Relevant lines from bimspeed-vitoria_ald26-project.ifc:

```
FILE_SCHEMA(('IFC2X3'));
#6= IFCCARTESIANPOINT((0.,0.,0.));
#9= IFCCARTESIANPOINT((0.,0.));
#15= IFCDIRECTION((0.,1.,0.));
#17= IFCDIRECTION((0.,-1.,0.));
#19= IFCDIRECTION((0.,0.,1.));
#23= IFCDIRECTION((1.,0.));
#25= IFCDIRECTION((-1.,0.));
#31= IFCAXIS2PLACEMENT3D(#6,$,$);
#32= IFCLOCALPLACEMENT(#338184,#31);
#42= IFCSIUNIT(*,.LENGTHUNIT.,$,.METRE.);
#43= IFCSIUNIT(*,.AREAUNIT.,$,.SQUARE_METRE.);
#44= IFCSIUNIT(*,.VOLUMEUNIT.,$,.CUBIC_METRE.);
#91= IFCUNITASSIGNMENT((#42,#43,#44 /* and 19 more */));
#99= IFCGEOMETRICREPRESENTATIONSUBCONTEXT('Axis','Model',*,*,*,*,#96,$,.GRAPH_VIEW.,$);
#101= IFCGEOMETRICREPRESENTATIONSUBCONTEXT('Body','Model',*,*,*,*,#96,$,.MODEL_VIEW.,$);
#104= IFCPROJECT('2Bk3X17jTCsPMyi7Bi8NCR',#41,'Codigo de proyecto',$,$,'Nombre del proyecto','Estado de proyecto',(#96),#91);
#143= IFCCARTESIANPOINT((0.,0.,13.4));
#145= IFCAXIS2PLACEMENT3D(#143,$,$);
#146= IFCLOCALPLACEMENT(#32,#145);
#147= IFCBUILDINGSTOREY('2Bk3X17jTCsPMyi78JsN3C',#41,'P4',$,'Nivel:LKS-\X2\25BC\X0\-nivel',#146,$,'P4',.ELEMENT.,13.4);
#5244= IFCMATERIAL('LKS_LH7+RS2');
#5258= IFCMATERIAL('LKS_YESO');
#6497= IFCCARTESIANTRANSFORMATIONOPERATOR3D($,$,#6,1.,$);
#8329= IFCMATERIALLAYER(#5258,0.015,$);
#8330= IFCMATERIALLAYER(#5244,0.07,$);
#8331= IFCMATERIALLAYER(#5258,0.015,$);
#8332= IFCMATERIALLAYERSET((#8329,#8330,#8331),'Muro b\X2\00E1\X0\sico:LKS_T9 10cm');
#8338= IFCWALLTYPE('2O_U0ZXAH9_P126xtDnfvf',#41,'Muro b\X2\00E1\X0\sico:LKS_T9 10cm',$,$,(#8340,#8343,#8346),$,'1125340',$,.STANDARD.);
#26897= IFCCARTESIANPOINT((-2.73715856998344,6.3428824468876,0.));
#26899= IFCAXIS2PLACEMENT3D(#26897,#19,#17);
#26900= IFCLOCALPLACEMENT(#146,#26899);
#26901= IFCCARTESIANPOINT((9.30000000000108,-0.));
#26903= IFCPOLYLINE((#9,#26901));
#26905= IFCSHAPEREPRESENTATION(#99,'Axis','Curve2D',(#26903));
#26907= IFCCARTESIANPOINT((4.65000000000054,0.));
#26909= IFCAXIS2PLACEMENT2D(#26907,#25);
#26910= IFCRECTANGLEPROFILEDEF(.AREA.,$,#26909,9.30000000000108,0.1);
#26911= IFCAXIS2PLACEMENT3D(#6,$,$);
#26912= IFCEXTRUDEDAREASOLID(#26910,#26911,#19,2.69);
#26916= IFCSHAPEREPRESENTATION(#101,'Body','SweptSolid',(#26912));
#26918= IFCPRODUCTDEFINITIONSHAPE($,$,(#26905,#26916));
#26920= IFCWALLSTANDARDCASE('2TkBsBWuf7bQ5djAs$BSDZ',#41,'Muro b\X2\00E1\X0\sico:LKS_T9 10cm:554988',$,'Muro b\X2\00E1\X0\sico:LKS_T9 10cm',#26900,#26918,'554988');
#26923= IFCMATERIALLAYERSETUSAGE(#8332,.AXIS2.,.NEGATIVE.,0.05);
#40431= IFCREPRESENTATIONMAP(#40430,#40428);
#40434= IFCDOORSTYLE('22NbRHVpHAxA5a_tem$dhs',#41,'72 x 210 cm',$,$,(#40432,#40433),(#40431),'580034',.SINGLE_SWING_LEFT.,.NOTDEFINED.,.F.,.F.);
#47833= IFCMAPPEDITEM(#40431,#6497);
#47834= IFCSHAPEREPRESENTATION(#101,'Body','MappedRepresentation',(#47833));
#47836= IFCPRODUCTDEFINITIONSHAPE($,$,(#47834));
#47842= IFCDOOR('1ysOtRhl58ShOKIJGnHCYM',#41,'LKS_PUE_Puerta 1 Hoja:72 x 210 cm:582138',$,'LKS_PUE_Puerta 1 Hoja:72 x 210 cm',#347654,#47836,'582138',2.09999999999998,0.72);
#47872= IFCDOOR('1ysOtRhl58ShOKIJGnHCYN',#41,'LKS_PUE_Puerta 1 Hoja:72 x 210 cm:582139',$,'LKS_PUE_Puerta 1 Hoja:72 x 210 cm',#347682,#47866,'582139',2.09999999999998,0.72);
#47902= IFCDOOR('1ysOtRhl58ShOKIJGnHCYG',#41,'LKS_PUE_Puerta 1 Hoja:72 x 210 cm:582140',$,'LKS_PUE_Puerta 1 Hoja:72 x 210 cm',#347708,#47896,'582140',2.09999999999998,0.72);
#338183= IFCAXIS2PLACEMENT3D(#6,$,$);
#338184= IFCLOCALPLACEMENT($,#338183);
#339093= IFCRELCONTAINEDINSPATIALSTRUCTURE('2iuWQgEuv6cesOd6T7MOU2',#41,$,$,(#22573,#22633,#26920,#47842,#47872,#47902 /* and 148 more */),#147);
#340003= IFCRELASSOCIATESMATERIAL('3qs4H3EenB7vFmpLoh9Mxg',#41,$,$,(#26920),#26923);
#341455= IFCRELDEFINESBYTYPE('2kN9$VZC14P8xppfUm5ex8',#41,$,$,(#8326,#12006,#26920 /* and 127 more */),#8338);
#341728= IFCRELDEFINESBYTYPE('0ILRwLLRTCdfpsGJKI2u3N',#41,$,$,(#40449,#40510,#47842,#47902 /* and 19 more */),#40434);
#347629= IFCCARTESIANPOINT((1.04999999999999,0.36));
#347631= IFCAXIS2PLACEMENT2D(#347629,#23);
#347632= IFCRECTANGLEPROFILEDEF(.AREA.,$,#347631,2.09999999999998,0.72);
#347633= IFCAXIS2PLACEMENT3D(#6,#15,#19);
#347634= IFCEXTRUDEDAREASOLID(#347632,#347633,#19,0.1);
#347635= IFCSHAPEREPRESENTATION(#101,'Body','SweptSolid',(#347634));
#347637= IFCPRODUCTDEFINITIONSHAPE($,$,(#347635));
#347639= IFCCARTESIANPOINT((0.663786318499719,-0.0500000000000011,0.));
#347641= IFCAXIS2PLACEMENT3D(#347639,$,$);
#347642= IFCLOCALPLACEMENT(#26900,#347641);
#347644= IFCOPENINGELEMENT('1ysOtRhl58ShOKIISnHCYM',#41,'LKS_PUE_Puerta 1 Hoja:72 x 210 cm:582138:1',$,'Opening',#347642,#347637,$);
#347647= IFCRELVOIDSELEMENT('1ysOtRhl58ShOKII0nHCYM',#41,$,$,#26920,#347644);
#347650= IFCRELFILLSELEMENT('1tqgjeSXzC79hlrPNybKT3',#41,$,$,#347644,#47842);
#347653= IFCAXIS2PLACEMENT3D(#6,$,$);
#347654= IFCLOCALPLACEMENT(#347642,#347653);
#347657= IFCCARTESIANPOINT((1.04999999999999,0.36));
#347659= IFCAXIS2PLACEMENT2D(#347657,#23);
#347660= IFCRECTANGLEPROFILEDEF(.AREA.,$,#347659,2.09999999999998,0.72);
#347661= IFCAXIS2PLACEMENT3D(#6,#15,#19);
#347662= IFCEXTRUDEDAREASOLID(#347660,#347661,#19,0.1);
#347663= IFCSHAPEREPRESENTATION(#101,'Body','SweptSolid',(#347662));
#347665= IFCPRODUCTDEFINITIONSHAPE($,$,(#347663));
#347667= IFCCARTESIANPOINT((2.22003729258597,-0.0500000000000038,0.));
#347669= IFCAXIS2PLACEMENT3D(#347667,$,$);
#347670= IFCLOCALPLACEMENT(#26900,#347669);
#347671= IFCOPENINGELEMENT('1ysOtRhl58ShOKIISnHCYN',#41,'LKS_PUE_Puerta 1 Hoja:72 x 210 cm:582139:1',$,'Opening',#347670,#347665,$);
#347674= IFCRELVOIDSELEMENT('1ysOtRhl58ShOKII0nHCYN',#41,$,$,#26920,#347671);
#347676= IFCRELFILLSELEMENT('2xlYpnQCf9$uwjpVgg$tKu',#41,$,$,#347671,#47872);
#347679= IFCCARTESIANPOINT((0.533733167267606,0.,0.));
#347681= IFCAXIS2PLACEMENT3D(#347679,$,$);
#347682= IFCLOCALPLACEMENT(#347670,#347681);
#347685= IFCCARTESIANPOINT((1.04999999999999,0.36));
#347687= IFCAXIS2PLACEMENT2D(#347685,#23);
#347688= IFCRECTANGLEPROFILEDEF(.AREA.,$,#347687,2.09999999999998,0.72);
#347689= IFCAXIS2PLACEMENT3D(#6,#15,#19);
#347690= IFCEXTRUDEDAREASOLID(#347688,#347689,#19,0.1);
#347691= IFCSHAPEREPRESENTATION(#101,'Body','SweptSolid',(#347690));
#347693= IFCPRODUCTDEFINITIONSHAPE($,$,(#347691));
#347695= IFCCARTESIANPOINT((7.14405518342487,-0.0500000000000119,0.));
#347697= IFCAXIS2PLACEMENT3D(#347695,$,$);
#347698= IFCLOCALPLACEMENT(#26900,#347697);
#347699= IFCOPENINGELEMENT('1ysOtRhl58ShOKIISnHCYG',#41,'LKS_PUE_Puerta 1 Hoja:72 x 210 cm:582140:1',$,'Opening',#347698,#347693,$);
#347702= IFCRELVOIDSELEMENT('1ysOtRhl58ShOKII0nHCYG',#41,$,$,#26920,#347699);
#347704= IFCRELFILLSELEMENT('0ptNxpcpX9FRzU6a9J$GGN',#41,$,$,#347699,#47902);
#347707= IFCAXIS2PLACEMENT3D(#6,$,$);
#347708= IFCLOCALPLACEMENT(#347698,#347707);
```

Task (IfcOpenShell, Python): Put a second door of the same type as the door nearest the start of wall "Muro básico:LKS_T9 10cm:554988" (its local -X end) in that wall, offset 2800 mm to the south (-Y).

```python
import ifcopenshell
import ifcopenshell.api.feature
import ifcopenshell.api.geometry
import ifcopenshell.api.root
import ifcopenshell.geom
import ifcopenshell.util.element
import ifcopenshell.util.placement
import ifcopenshell.util.shape

model = ifcopenshell.open("bimspeed-vitoria_ald26-project.ifc")
settings = ifcopenshell.geom.settings()


def volume(element):
    """Net volume in cubic metres, openings subtracted."""
    shape = ifcopenshell.geom.create_shape(settings, element)
    return ifcopenshell.util.shape.get_volume(shape.geometry)


def reuse_history(source, copy):
    """copy_class also copies each property set's owner history, people and application; keep the originals."""
    for rel in copy.IsDefinedBy:
        if rel.is_a("IfcRelDefinesByProperties") and (history := rel.RelatingPropertyDefinition.OwnerHistory):
            rel.RelatingPropertyDefinition.OwnerHistory = source.OwnerHistory
            ifcopenshell.util.element.remove_deep2(model, history)


door = model.by_id(47842)
opening = door.FillsVoids[0].RelatingOpeningElement
wall = opening.VoidsElements[0].RelatingBuildingElement
before = volume(wall)
shift = ifcopenshell.util.placement.get_local_placement(wall.ObjectPlacement)[:3, 0] * 2.8

# copy_class copies the void relationship, type, container and properties, but no geometry.
new_opening = ifcopenshell.api.root.copy_class(model, product=opening)
new_opening.Representation = ifcopenshell.util.element.copy_deep(
    model, opening.Representation, exclude=["IfcGeometricRepresentationContext", "IfcRepresentationMap"]
)
new_opening.Name = "LKS_PUE_Puerta 1 Hoja:72 x 210 cm"
new_door = ifcopenshell.api.root.copy_class(model, product=door)
new_door.Representation = ifcopenshell.util.element.copy_deep(
    model, door.Representation, exclude=["IfcGeometricRepresentationContext", "IfcRepresentationMap"]
)
new_door.Name = "LKS_PUE_Puerta 1 Hoja:72 x 210 cm"
new_door.Tag = None
reuse_history(door, new_door)
fills = ifcopenshell.api.feature.add_filling(model, opening=new_opening, element=new_door)
fills.OwnerHistory = new_door.OwnerHistory  # required in IFC2X3

for old, new in ((opening, new_opening), (door, new_door)):
    matrix = ifcopenshell.util.placement.get_local_placement(old.ObjectPlacement)
    matrix[:3, 3] += shift
    ifcopenshell.api.geometry.edit_object_placement(model, product=new, matrix=matrix, is_si=False)

after = volume(wall)

print(f"wall volume {before:.3f} -> {after:.3f} m3")

model.write("bimspeed-vitoria_ald26-project_edited.ifc")
```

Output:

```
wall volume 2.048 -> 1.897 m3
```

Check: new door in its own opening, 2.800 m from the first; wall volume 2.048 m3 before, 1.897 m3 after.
